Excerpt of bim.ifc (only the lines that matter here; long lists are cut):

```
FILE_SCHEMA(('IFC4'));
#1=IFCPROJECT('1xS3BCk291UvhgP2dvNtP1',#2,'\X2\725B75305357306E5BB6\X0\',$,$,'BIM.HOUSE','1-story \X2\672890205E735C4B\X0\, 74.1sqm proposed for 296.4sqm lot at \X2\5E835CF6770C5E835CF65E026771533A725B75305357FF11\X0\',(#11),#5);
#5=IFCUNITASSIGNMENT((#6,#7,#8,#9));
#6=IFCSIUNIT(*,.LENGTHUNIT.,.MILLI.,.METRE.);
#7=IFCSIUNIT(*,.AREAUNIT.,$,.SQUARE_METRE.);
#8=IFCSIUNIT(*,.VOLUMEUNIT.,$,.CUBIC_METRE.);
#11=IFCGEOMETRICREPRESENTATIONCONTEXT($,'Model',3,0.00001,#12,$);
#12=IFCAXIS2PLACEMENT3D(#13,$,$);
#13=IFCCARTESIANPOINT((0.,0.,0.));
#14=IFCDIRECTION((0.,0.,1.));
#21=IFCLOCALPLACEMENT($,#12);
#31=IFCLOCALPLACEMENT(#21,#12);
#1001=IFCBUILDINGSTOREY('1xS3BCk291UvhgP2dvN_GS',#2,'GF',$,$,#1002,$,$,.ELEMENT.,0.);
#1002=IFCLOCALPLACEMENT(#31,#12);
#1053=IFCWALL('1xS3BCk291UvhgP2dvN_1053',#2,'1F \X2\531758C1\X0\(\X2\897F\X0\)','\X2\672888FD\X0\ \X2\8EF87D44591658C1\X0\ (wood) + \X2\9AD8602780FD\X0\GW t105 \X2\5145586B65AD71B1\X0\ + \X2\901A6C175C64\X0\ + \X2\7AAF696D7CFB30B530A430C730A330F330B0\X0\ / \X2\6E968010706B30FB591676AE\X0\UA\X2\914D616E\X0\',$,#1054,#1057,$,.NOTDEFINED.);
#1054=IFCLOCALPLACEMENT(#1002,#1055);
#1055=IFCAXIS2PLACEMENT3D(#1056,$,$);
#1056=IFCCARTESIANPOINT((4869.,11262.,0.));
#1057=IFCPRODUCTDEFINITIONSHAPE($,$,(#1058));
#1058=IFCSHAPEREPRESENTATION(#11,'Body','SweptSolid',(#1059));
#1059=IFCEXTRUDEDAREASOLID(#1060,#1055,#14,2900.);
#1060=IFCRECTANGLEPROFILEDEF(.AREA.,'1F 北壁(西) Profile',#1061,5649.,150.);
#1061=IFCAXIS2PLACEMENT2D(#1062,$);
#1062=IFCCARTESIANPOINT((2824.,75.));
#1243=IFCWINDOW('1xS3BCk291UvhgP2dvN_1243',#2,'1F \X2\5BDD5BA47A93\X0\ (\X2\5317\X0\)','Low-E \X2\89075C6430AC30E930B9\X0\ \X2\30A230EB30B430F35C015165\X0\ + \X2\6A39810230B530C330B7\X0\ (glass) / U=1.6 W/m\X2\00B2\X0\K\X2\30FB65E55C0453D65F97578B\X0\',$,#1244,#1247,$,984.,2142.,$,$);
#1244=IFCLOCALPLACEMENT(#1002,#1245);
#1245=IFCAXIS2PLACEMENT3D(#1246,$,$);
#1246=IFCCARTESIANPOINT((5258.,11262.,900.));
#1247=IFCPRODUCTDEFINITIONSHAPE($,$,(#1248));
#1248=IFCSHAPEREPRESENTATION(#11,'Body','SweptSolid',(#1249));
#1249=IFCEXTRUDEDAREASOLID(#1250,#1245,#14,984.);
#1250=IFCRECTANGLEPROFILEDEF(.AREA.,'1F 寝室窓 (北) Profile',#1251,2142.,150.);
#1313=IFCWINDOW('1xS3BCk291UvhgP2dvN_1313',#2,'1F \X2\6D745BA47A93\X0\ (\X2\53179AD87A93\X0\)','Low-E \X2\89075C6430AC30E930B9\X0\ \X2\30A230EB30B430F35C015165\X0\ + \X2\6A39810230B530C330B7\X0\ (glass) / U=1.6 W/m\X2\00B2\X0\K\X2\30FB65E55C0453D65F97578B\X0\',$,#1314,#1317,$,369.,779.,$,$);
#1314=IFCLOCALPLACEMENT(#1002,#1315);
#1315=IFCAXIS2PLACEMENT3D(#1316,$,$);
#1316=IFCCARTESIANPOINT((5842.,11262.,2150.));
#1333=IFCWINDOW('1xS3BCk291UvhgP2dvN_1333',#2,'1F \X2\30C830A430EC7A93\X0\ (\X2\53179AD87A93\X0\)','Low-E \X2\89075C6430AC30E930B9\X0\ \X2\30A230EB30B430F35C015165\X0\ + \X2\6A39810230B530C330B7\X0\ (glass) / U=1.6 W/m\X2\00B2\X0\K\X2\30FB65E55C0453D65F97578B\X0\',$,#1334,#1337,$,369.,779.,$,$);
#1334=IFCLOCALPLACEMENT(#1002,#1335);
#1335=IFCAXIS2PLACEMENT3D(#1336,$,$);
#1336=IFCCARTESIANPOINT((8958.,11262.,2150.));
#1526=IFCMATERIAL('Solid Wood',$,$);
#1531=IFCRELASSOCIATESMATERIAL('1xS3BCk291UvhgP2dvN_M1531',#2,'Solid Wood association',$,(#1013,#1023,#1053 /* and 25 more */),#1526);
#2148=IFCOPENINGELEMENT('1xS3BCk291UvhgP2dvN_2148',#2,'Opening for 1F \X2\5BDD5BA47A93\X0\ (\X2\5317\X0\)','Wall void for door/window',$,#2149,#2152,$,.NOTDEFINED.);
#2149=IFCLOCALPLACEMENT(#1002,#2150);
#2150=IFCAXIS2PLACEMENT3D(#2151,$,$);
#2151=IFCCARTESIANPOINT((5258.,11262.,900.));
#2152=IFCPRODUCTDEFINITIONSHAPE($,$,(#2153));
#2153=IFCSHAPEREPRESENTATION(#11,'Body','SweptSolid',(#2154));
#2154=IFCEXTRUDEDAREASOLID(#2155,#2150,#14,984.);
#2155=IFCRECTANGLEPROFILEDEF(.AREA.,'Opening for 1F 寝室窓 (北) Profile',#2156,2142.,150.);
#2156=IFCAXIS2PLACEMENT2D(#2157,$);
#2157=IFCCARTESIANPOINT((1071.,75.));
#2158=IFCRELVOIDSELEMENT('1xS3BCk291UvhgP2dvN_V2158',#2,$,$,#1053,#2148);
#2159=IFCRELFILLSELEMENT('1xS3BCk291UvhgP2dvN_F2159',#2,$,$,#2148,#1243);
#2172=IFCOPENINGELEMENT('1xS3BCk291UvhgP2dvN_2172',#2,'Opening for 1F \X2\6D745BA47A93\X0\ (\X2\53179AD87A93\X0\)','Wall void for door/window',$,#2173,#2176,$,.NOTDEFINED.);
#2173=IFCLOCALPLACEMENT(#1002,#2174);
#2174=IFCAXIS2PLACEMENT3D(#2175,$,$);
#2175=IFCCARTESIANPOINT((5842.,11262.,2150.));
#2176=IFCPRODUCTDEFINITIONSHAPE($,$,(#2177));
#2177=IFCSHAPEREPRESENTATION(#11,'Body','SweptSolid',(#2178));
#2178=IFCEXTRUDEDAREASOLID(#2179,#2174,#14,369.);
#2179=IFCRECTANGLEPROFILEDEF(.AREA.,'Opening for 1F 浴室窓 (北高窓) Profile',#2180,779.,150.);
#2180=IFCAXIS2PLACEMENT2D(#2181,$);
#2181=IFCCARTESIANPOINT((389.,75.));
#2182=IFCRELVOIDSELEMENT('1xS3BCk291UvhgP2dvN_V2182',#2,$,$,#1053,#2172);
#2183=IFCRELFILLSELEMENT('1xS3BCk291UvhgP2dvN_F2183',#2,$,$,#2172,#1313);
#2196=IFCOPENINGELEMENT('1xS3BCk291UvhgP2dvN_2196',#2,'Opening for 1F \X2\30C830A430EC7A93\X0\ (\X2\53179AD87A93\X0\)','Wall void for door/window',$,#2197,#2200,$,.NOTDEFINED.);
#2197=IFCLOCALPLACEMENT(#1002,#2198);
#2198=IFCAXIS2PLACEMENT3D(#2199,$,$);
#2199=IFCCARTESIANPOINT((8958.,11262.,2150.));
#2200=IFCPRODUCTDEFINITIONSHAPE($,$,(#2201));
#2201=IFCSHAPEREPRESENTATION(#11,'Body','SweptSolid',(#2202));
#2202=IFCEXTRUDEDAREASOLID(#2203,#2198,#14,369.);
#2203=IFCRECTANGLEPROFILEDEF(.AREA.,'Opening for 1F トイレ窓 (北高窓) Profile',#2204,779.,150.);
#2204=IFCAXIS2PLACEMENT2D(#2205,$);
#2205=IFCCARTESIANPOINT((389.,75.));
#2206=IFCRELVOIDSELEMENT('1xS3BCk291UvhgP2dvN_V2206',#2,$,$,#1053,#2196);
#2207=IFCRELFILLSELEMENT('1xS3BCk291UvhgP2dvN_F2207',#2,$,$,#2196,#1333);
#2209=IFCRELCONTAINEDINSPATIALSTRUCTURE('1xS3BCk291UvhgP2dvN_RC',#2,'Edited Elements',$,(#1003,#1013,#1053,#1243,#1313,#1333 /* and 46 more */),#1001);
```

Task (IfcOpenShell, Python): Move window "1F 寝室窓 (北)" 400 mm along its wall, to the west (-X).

```python
import ifcopenshell
import ifcopenshell.api.geometry
import ifcopenshell.util.placement
import ifcopenshell.util.unit

model = ifcopenshell.open("bim.ifc")
unit_scale = ifcopenshell.util.unit.calculate_unit_scale(model)

window = model.by_guid("1xS3BCk291UvhgP2dvN_1243")
opening = window.FillsVoids[0].RelatingOpeningElement
wall = opening.VoidsElements[0].RelatingBuildingElement

wall_matrix = ifcopenshell.util.placement.get_local_placement(wall.ObjectPlacement)
shift = wall_matrix[:3, 0] * -0.4 / unit_scale
before = ifcopenshell.util.placement.get_local_placement(window.ObjectPlacement)[:3, 3].copy()

# The window is not placed relative to its opening, so move both.
for product in (opening, window):
    matrix = ifcopenshell.util.placement.get_local_placement(product.ObjectPlacement)
    matrix[:3, 3] += shift
    ifcopenshell.api.geometry.edit_object_placement(model, product=product, matrix=matrix, is_si=False)

after = ifcopenshell.util.placement.get_local_placement(window.ObjectPlacement)[:3, 3]
print("window moved by", (after - before).round(3) + 0.0)

model.write("bim_rev.ifc")
```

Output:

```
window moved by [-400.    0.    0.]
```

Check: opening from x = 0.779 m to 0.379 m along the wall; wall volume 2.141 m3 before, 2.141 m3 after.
